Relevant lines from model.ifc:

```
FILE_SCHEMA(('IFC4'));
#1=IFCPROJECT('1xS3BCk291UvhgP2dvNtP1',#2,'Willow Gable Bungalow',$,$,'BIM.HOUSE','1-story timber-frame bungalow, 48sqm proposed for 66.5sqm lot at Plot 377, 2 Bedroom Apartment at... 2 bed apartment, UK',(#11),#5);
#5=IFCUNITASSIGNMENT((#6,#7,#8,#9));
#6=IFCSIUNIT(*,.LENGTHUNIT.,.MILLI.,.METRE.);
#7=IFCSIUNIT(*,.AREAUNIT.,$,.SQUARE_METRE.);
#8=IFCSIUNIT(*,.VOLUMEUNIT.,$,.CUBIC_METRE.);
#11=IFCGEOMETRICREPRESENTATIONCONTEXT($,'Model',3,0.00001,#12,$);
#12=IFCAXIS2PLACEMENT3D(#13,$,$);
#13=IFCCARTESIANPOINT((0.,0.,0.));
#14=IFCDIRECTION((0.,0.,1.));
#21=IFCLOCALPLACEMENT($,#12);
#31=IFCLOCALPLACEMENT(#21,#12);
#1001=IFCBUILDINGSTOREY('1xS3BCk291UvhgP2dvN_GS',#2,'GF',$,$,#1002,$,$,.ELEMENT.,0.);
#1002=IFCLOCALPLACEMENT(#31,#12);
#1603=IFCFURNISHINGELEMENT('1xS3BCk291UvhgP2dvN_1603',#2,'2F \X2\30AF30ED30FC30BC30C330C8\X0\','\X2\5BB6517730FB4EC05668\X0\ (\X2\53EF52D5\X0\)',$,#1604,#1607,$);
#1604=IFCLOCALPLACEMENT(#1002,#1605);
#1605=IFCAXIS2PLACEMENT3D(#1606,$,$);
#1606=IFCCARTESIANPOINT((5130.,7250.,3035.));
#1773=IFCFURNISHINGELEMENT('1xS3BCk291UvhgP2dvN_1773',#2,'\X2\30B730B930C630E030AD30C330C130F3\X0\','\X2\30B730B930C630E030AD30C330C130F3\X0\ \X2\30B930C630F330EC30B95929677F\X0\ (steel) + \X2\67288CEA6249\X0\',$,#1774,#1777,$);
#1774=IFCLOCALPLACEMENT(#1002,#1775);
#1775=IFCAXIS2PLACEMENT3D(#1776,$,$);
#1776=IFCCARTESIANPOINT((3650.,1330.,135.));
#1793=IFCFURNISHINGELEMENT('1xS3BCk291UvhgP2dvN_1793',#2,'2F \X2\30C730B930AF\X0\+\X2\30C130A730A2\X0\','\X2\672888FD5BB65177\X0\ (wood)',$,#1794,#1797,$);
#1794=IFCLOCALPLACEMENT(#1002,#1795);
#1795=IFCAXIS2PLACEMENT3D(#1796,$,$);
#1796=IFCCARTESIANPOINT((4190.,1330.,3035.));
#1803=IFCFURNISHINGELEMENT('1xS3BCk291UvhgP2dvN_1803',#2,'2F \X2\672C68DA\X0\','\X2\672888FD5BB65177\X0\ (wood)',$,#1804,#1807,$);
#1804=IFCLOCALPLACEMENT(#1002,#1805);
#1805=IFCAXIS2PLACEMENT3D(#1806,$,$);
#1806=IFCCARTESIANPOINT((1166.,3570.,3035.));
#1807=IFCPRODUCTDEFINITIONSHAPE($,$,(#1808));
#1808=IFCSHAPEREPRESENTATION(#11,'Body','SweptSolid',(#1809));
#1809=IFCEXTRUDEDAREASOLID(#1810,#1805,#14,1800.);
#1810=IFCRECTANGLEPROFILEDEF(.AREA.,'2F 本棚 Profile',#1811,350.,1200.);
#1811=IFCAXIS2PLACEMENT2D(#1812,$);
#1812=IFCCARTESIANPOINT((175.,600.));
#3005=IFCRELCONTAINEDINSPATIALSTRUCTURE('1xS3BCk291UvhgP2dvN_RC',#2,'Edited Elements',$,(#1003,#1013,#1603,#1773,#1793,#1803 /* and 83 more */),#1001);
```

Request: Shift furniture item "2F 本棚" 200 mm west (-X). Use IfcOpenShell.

```python
import ifcopenshell
import ifcopenshell.api.geometry
import ifcopenshell.util.placement

model = ifcopenshell.open("model.ifc")

item = model.by_guid("1xS3BCk291UvhgP2dvN_1803")
matrix = ifcopenshell.util.placement.get_local_placement(item.ObjectPlacement)
matrix[0, 3] -= 200.0
ifcopenshell.api.geometry.edit_object_placement(model, product=item, matrix=matrix, is_si=False)

print(ifcopenshell.util.placement.get_local_placement(item.ObjectPlacement).round(3) + 0.0)

model.write("model_edited.ifc")
```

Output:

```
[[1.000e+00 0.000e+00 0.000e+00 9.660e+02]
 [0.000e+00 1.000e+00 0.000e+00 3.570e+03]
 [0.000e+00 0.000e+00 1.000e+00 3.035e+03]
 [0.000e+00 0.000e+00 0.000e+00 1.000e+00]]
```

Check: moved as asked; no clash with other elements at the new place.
